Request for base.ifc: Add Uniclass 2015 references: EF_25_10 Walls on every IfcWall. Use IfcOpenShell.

First a look at what the model holds.

```python
import ifcopenshell

model = ifcopenshell.open("base.ifc")
print(model.schema)
print("classifications:", [c.Name for c in model.by_type("IfcClassification")])
for ifc_class in ("IfcDoor", "IfcRoof", "IfcStair", "IfcWall", "IfcWindow"):
    print(ifc_class, len(model.by_type(ifc_class)))
```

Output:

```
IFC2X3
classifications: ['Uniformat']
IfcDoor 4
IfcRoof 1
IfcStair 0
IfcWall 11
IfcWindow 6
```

```python
import ifcopenshell
import ifcopenshell.api.classification

model = ifcopenshell.open("base.ifc")

# IFC2X3 requires Source and Edition and has no link from the project to the system.
system = model.create_entity("IfcClassification", Source="NBS", Edition="2015", Name="Uniclass 2015")

codes = {
    "IfcWall": ("EF_25_10", "Walls"),
}
for ifc_class, (code, name) in codes.items():
    products = model.by_type(ifc_class)
    ifcopenshell.api.classification.add_reference(
        model, products=products, classification=system, identification=code, name=name
    )
    print(code, len(products))

model.write("base-out.ifc")
```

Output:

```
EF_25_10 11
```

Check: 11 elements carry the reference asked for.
